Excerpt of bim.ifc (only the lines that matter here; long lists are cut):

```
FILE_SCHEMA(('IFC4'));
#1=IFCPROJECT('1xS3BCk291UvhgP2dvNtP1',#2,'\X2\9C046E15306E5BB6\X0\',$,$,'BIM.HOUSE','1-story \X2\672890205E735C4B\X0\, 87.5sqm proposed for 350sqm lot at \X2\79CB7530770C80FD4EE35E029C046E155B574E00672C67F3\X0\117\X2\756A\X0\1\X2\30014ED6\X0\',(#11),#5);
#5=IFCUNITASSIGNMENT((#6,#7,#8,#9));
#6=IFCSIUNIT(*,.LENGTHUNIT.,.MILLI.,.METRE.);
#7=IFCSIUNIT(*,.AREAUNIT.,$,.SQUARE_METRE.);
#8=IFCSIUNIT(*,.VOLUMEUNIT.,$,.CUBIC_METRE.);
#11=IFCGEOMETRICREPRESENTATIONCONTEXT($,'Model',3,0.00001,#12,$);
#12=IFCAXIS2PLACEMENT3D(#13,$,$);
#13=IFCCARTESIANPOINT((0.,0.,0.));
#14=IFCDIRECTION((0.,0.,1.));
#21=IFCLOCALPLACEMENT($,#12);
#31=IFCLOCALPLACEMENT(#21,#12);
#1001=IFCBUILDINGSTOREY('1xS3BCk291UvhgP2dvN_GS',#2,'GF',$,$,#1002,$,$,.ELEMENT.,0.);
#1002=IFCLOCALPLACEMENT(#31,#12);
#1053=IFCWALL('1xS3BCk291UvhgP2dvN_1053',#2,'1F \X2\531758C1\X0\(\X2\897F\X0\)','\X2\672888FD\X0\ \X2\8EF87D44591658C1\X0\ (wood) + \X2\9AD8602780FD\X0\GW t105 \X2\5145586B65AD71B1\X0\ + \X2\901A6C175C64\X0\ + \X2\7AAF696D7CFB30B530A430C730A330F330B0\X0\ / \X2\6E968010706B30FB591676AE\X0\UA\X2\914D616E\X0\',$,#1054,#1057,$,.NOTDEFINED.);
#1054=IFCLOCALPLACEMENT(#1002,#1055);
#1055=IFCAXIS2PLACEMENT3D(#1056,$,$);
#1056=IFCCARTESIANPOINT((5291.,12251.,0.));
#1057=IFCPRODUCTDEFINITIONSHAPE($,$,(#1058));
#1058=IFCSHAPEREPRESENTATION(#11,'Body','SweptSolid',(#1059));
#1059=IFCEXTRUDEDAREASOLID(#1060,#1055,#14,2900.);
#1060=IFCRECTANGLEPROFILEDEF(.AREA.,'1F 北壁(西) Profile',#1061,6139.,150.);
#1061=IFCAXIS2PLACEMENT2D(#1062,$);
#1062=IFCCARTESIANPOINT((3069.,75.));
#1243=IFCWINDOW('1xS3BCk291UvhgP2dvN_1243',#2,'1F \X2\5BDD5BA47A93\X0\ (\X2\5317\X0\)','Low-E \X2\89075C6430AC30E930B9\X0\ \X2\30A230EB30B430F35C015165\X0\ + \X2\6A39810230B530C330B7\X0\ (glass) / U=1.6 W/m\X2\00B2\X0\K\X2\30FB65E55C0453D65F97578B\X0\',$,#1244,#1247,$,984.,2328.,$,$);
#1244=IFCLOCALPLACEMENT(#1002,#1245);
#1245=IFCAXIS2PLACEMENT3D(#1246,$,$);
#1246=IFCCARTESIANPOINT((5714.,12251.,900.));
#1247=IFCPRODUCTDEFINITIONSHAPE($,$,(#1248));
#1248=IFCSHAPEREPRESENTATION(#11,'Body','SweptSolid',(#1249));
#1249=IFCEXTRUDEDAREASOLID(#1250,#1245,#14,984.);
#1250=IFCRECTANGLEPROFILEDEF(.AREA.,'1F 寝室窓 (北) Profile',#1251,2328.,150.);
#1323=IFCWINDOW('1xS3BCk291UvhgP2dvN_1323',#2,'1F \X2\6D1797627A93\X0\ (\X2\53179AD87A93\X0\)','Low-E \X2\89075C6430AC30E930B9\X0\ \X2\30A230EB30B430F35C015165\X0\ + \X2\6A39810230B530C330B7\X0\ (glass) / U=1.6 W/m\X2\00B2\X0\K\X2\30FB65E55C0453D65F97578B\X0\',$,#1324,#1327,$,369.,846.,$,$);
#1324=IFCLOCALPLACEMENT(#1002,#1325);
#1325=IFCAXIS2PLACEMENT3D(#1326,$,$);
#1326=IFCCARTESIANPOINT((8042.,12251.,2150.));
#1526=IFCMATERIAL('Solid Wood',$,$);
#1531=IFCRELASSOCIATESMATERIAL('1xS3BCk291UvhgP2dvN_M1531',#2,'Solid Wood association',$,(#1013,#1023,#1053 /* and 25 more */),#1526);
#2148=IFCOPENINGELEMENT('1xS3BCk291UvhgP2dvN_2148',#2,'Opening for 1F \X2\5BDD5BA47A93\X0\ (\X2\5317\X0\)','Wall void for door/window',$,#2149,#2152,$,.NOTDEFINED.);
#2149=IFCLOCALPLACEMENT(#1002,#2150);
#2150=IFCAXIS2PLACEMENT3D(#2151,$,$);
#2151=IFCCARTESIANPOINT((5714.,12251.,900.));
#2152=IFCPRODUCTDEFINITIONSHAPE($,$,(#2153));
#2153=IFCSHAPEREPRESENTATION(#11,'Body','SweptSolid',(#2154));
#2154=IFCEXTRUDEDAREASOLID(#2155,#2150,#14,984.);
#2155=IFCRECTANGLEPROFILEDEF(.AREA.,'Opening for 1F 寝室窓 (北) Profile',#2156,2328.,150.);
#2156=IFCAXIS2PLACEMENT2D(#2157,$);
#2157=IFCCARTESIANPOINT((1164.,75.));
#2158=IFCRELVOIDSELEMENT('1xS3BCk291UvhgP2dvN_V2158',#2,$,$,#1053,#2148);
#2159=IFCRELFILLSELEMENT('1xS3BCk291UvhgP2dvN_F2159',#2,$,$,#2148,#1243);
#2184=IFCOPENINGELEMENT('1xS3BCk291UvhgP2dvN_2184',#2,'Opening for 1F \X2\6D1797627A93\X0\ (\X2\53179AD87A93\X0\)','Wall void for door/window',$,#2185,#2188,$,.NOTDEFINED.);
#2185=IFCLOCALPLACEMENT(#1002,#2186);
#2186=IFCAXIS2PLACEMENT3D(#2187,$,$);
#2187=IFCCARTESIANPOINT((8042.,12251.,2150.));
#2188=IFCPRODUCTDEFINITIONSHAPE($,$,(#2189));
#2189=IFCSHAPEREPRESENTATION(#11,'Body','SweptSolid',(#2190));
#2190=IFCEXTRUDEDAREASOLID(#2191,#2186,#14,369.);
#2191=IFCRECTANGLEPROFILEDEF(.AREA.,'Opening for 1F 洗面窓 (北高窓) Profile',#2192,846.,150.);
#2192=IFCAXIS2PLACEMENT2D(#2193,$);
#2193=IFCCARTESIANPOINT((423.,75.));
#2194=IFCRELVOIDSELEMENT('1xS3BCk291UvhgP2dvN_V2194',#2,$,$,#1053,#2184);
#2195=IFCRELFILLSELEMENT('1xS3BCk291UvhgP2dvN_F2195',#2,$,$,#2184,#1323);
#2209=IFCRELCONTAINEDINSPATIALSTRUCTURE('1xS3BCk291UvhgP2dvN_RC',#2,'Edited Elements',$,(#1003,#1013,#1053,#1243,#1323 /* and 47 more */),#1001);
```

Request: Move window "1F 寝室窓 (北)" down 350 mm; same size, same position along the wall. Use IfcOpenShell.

```python
import numpy as np
import ifcopenshell
import ifcopenshell.api.geometry
import ifcopenshell.util.placement
import ifcopenshell.util.unit

model = ifcopenshell.open("bim.ifc")
unit_scale = ifcopenshell.util.unit.calculate_unit_scale(model)

window = model.by_guid("1xS3BCk291UvhgP2dvN_1243")
opening = window.FillsVoids[0].RelatingOpeningElement
dz = -0.35 / unit_scale

shift = np.array([0.0, 0.0, dz])
# The window is not placed relative to its opening, so move both.
for product in (opening, window):
    matrix = ifcopenshell.util.placement.get_local_placement(product.ObjectPlacement)
    matrix[:3, 3] += shift
    ifcopenshell.api.geometry.edit_object_placement(model, product=product, matrix=matrix, is_si=False)

print(f"moved by {dz * unit_scale:+.3f} m")

model.write("bim_updated.ifc")
```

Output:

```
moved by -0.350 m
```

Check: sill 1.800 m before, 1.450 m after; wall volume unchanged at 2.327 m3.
